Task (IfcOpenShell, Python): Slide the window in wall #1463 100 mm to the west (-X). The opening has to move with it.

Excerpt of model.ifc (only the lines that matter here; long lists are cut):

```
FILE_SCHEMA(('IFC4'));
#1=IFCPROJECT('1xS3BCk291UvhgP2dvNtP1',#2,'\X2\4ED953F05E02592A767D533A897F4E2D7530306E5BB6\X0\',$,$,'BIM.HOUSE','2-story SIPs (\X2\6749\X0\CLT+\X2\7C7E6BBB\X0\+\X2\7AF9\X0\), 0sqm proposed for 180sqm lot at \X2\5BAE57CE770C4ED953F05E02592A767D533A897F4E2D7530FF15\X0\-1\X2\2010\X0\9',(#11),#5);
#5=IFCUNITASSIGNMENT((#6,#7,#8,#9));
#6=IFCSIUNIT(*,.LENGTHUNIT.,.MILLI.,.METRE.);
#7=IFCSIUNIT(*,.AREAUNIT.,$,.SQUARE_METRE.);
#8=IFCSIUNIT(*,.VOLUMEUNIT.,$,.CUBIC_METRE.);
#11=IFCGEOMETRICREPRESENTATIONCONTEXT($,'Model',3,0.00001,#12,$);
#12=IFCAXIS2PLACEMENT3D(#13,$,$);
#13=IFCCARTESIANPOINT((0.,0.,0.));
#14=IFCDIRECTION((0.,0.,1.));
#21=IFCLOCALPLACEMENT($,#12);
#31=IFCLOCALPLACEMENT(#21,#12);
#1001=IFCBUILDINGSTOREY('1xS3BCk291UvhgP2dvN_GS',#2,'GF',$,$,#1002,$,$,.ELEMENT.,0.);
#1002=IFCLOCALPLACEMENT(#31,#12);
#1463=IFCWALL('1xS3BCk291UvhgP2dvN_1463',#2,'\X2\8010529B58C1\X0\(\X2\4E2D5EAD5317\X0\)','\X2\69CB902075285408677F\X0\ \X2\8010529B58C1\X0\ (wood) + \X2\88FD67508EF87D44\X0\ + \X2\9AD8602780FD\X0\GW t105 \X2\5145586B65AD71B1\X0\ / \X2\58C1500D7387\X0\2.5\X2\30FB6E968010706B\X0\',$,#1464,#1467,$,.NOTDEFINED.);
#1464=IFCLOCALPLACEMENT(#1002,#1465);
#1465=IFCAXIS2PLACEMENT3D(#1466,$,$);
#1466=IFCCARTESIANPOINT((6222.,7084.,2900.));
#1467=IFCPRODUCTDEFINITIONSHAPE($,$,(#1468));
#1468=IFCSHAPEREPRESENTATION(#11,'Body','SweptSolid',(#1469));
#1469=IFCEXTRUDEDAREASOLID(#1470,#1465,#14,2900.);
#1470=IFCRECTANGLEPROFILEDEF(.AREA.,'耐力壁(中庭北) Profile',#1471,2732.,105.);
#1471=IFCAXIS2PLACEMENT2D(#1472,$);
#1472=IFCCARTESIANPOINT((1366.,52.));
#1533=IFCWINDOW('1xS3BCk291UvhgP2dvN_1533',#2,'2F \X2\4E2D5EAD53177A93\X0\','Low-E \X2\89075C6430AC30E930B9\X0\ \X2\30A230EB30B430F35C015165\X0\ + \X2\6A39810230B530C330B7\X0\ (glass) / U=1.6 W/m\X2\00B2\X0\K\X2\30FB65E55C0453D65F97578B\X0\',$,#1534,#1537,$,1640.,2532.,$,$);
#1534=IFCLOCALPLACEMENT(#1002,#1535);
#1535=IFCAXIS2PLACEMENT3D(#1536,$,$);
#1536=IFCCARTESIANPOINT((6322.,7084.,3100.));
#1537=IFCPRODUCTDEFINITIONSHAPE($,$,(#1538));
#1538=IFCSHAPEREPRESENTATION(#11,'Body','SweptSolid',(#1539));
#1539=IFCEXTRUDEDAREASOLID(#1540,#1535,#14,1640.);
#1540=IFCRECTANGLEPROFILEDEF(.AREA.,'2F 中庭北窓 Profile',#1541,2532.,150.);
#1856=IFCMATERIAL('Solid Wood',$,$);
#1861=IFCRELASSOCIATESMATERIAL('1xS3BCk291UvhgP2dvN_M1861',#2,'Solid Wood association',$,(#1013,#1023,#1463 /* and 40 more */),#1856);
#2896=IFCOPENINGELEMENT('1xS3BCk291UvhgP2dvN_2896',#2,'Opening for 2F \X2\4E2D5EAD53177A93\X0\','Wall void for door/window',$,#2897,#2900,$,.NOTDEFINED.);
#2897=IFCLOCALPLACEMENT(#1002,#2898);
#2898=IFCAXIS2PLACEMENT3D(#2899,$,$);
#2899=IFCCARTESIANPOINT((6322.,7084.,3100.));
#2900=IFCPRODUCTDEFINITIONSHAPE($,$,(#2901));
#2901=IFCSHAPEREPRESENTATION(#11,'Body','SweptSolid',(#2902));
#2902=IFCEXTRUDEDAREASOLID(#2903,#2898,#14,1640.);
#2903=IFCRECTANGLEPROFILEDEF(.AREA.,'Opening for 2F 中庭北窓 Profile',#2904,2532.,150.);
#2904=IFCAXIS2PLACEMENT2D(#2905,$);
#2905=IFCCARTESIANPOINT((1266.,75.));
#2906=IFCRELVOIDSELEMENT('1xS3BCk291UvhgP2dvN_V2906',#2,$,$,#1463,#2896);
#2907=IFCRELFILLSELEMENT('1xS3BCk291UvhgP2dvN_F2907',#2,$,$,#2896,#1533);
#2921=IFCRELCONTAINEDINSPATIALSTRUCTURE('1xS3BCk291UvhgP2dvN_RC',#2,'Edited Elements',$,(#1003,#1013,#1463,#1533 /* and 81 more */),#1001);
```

```python
import ifcopenshell
import ifcopenshell.api.geometry
import ifcopenshell.util.placement
import ifcopenshell.util.unit

model = ifcopenshell.open("model.ifc")
unit_scale = ifcopenshell.util.unit.calculate_unit_scale(model)

window = model.by_id(1533)
opening = window.FillsVoids[0].RelatingOpeningElement
wall = opening.VoidsElements[0].RelatingBuildingElement

wall_matrix = ifcopenshell.util.placement.get_local_placement(wall.ObjectPlacement)
shift = wall_matrix[:3, 0] * -0.1 / unit_scale
before = ifcopenshell.util.placement.get_local_placement(window.ObjectPlacement)[:3, 3].copy()

# The window is not placed relative to its opening, so move both.
for product in (opening, window):
    matrix = ifcopenshell.util.placement.get_local_placement(product.ObjectPlacement)
    matrix[:3, 3] += shift
    ifcopenshell.api.geometry.edit_object_placement(model, product=product, matrix=matrix, is_si=False)

after = ifcopenshell.util.placement.get_local_placement(window.ObjectPlacement)[:3, 3]
print("window moved by", (after - before).round(3) + 0.0)

model.write("model-out.ifc")
```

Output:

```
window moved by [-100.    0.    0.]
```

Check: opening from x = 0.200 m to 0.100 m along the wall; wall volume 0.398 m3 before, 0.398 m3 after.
